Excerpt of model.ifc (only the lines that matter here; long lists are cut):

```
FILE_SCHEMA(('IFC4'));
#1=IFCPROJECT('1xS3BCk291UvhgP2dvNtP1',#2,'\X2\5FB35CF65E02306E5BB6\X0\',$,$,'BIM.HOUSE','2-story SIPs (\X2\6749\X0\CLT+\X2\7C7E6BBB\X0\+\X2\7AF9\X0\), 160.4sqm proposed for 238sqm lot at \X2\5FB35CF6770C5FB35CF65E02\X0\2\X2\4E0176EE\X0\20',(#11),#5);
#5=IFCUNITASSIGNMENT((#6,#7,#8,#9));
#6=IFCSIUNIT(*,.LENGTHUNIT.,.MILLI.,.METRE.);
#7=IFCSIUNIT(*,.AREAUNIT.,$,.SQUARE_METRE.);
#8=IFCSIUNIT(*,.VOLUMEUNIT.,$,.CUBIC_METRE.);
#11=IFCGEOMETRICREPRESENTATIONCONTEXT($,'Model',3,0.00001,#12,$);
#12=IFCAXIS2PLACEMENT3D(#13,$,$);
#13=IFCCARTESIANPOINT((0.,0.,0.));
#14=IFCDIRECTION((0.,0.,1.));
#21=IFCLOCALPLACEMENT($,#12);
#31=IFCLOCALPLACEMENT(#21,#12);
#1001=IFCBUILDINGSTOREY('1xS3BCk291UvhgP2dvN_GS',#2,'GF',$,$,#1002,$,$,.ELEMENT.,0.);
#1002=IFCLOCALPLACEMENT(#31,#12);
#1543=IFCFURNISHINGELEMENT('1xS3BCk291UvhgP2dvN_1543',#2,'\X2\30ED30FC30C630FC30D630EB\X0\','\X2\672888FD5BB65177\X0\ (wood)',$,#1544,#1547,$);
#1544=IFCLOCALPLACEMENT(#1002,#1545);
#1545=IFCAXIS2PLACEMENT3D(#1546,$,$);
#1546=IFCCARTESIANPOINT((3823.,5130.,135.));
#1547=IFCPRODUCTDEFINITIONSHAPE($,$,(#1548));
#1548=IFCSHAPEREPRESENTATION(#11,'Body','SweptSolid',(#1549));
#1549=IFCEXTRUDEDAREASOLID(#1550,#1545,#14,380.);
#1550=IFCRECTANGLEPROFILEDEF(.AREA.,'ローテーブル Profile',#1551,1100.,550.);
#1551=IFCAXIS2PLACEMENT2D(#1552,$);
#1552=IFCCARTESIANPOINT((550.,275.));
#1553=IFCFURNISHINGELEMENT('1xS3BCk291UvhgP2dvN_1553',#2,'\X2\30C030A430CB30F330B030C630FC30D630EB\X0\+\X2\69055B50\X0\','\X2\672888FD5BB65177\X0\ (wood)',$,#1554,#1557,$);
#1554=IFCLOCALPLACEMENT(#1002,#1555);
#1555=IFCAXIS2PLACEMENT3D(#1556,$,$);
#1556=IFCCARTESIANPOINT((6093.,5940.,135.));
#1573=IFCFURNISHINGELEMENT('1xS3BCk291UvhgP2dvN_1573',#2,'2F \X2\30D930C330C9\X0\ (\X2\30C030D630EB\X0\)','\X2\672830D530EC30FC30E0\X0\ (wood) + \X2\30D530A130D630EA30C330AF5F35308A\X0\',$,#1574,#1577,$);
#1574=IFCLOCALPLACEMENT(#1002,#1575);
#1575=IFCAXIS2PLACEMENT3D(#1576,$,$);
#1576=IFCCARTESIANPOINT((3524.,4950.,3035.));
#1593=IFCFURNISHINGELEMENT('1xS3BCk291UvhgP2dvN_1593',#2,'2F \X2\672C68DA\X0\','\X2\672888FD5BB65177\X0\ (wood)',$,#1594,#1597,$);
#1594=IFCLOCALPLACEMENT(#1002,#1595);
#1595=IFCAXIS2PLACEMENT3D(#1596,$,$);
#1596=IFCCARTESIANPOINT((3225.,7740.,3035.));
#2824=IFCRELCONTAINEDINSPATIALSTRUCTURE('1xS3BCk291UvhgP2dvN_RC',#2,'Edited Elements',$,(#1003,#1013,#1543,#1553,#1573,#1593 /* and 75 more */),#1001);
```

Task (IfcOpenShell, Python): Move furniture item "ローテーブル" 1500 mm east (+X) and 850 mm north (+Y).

```python
import ifcopenshell
import ifcopenshell.api.geometry
import ifcopenshell.util.placement

model = ifcopenshell.open("model.ifc")

item = model.by_guid("1xS3BCk291UvhgP2dvN_1543")
matrix = ifcopenshell.util.placement.get_local_placement(item.ObjectPlacement)
matrix[0, 3] += 1500.0
matrix[1, 3] += 850.0
ifcopenshell.api.geometry.edit_object_placement(model, product=item, matrix=matrix, is_si=False)

print(ifcopenshell.util.placement.get_local_placement(item.ObjectPlacement).round(3) + 0.0)

model.write("model_rev.ifc")
```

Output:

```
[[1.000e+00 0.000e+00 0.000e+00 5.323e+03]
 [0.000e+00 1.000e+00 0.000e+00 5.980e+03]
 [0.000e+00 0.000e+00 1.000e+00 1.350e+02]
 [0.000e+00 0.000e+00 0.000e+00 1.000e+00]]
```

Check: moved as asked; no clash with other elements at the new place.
